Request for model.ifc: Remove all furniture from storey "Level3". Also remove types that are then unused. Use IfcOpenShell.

First a look at what the model holds.

```python
import ifcopenshell
import ifcopenshell.util.element

model = ifcopenshell.open("model.ifc")
print(model.schema)
storey = next(s for s in model.by_type("IfcBuildingStorey") if s.Name == "Level3")
furniture = [e for e in ifcopenshell.util.element.get_decomposition(storey) if e.is_a("IfcFurnishingElement")]
seen = {}
for e in furniture:
    element_type = ifcopenshell.util.element.get_type(e)
    name = element_type.Name if element_type not in (None, e) else None
    seen[name] = seen.get(name, 0) + 1
for name, count in sorted(seen.items(), key=str):
    print(count, "x", name)
```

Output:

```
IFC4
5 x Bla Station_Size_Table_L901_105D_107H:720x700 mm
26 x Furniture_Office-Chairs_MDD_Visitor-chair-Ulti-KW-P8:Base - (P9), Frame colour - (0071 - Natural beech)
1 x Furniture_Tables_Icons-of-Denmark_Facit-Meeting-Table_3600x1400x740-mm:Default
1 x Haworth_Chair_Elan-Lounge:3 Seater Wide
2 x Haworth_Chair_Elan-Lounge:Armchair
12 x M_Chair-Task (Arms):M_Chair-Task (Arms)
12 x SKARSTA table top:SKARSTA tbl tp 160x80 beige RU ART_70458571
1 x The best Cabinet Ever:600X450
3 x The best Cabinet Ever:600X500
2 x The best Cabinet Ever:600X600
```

```python
import ifcopenshell
import ifcopenshell.api.root
import ifcopenshell.util.element

model = ifcopenshell.open("model.ifc")

storey = next(s for s in model.by_type("IfcBuildingStorey") if s.Name == "Level3")
furniture = [e for e in ifcopenshell.util.element.get_decomposition(storey) if e.is_a("IfcFurnishingElement")]
types = {ifcopenshell.util.element.get_type(e) for e in furniture} - {None, *furniture}

for e in furniture:
    ifcopenshell.api.root.remove_product(model, product=e)
print(len(furniture), "removed")

unused = [t for t in types if not ifcopenshell.util.element.get_types(t)]
for t in unused:
    ifcopenshell.api.root.remove_product(model, product=t)
print(len(unused), "unused types removed")

model.write("model-out.ifc")
```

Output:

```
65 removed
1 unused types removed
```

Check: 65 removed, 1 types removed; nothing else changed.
